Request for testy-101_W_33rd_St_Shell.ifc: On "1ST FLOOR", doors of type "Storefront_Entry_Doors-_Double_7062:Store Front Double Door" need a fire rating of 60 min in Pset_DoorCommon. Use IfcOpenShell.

First a look at what the model holds.

```python
import ifcopenshell
import ifcopenshell.util.element

model = ifcopenshell.open("testy-101_W_33rd_St_Shell.ifc")
print(model.schema)
storey = next(s for s in model.by_type("IfcBuildingStorey") if s.Name == "1ST FLOOR")
doors = [e for e in ifcopenshell.util.element.get_decomposition(storey) if e.is_a("IfcDoor")]
seen = {}
for e in doors:
    element_type = ifcopenshell.util.element.get_type(e)
    key = (element_type.Name if element_type != e and element_type else None, ifcopenshell.util.element.get_pset(e, "Pset_DoorCommon", "FireRating"))
    seen[key] = seen.get(key, 0) + 1
for (name, value), count in sorted(seen.items(), key=str):
    print(count, "x", name, "|", value)
```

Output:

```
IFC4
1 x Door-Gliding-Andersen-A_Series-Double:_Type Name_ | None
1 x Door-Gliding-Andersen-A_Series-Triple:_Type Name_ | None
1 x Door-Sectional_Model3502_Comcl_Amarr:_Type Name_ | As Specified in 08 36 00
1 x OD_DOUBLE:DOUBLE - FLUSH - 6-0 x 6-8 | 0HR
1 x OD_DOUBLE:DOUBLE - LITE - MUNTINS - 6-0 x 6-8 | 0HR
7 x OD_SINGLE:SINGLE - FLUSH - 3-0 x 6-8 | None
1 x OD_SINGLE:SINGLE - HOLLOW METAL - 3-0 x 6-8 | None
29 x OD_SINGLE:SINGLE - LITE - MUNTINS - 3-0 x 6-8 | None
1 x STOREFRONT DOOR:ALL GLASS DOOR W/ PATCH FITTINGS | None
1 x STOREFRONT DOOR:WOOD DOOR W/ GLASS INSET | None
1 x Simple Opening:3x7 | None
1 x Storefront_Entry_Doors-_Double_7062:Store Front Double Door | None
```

```python
import ifcopenshell
import ifcopenshell.api.pset
import ifcopenshell.util.element

model = ifcopenshell.open("testy-101_W_33rd_St_Shell.ifc")

storey = next(s for s in model.by_type("IfcBuildingStorey") if s.Name == "1ST FLOOR")
doors = [e for e in ifcopenshell.util.element.get_decomposition(storey) if e.is_a("IfcDoor")]

count = 0
for e in doors:
    element_type = ifcopenshell.util.element.get_type(e)
    if element_type in (None, e) or element_type.Name != "Storefront_Entry_Doors-_Double_7062:Store Front Double Door":
        continue
    # add_pset returns the element's existing set when there is one.
    pset = ifcopenshell.api.pset.add_pset(model, product=e, name="Pset_DoorCommon")
    ifcopenshell.api.pset.edit_pset(model, pset=pset, properties={"FireRating": "60 min"})
    count += 1

print(count, "doors updated")

model.write("testy-101_W_33rd_St_Shell-out.ifc")
```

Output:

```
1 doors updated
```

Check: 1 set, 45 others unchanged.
